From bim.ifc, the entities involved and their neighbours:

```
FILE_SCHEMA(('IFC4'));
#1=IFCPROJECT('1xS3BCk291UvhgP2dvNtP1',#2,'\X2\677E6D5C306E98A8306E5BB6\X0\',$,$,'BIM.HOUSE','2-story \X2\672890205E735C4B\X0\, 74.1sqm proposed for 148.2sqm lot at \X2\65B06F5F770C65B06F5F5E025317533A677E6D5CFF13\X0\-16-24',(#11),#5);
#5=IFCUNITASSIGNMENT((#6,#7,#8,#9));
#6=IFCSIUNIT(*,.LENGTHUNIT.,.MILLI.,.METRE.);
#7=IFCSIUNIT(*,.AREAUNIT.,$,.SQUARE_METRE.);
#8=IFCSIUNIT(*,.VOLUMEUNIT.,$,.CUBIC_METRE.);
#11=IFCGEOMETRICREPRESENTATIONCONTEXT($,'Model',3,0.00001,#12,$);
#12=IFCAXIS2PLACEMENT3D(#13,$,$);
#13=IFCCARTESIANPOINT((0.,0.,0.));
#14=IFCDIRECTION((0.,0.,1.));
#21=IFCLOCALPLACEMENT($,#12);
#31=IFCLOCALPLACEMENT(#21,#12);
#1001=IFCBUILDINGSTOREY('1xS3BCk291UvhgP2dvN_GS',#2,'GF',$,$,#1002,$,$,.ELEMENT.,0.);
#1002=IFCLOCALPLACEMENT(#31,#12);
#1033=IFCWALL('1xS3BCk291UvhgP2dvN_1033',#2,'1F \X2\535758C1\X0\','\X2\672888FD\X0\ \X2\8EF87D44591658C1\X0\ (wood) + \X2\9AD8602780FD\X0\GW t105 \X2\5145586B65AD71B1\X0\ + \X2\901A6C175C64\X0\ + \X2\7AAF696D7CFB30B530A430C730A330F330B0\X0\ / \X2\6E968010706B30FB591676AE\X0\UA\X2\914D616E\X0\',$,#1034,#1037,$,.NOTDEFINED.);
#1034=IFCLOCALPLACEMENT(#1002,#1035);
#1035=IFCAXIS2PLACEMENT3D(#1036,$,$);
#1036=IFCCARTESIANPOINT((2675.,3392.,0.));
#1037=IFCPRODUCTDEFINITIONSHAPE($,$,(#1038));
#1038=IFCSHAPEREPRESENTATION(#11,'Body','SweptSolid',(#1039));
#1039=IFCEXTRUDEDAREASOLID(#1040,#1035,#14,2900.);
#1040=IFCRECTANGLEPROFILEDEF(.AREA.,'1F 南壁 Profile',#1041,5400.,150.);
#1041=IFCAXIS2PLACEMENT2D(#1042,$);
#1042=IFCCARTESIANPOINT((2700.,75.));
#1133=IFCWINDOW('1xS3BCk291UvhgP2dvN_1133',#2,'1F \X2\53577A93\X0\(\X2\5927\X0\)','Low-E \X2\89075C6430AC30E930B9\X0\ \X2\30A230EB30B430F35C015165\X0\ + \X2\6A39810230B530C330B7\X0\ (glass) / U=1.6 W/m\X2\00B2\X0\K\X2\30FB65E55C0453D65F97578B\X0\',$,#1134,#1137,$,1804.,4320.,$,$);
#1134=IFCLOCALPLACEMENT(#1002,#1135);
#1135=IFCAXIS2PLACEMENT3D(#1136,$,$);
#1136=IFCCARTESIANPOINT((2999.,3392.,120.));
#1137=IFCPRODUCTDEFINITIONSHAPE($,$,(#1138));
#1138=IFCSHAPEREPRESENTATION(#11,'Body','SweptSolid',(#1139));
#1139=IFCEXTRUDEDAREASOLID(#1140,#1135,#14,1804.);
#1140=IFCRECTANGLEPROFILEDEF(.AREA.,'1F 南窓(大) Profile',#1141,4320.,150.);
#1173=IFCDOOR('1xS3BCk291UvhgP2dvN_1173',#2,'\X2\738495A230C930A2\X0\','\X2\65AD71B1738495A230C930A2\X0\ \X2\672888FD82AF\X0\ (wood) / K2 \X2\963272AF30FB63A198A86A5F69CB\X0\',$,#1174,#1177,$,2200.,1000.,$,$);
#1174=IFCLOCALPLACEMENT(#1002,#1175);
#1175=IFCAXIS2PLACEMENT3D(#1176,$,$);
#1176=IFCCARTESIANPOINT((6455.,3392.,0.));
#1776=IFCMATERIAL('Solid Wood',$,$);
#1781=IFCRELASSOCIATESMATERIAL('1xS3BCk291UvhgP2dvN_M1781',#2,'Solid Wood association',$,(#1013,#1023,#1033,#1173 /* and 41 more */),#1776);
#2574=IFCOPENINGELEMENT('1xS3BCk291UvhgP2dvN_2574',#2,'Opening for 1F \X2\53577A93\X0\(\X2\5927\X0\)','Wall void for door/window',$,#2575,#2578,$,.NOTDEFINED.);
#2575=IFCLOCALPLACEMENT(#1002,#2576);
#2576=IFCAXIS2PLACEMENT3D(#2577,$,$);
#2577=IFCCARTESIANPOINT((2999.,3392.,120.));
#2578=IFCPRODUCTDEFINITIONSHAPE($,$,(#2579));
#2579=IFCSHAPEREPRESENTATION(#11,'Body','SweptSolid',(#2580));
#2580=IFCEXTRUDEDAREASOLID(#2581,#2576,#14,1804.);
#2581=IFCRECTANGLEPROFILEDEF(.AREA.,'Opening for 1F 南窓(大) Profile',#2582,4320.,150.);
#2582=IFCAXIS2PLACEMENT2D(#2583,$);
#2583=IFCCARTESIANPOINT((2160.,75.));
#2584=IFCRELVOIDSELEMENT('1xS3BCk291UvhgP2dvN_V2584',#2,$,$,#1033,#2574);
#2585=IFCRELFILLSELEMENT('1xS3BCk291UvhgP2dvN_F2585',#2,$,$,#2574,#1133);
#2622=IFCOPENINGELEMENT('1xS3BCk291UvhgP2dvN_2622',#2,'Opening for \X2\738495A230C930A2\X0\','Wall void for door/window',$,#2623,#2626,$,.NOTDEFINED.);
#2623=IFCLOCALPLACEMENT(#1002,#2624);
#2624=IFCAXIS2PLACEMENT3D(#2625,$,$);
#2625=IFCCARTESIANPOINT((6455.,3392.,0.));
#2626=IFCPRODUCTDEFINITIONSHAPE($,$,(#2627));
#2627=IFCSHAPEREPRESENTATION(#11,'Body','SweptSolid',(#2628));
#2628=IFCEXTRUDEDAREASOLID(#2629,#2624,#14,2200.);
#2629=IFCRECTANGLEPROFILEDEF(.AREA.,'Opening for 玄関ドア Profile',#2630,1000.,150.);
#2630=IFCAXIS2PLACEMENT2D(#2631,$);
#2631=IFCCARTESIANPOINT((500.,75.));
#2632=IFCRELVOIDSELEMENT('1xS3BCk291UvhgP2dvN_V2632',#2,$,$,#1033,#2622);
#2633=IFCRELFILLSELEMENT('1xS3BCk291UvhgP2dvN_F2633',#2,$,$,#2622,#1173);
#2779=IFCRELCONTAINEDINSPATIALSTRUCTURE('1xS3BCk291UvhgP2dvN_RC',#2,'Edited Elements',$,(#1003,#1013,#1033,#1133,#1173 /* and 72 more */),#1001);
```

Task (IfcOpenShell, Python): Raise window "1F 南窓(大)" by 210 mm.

```python
import numpy as np
import ifcopenshell
import ifcopenshell.api.geometry
import ifcopenshell.util.placement
import ifcopenshell.util.unit

model = ifcopenshell.open("bim.ifc")
unit_scale = ifcopenshell.util.unit.calculate_unit_scale(model)

window = model.by_guid("1xS3BCk291UvhgP2dvN_1133")
opening = window.FillsVoids[0].RelatingOpeningElement
dz = 0.21 / unit_scale

shift = np.array([0.0, 0.0, dz])
# The window is not placed relative to its opening, so move both.
for product in (opening, window):
    matrix = ifcopenshell.util.placement.get_local_placement(product.ObjectPlacement)
    matrix[:3, 3] += shift
    ifcopenshell.api.geometry.edit_object_placement(model, product=product, matrix=matrix, is_si=False)

print(f"moved by {dz * unit_scale:+.3f} m")

model.write("bim_updated.ifc")
```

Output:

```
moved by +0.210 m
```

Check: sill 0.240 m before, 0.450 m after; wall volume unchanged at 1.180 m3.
